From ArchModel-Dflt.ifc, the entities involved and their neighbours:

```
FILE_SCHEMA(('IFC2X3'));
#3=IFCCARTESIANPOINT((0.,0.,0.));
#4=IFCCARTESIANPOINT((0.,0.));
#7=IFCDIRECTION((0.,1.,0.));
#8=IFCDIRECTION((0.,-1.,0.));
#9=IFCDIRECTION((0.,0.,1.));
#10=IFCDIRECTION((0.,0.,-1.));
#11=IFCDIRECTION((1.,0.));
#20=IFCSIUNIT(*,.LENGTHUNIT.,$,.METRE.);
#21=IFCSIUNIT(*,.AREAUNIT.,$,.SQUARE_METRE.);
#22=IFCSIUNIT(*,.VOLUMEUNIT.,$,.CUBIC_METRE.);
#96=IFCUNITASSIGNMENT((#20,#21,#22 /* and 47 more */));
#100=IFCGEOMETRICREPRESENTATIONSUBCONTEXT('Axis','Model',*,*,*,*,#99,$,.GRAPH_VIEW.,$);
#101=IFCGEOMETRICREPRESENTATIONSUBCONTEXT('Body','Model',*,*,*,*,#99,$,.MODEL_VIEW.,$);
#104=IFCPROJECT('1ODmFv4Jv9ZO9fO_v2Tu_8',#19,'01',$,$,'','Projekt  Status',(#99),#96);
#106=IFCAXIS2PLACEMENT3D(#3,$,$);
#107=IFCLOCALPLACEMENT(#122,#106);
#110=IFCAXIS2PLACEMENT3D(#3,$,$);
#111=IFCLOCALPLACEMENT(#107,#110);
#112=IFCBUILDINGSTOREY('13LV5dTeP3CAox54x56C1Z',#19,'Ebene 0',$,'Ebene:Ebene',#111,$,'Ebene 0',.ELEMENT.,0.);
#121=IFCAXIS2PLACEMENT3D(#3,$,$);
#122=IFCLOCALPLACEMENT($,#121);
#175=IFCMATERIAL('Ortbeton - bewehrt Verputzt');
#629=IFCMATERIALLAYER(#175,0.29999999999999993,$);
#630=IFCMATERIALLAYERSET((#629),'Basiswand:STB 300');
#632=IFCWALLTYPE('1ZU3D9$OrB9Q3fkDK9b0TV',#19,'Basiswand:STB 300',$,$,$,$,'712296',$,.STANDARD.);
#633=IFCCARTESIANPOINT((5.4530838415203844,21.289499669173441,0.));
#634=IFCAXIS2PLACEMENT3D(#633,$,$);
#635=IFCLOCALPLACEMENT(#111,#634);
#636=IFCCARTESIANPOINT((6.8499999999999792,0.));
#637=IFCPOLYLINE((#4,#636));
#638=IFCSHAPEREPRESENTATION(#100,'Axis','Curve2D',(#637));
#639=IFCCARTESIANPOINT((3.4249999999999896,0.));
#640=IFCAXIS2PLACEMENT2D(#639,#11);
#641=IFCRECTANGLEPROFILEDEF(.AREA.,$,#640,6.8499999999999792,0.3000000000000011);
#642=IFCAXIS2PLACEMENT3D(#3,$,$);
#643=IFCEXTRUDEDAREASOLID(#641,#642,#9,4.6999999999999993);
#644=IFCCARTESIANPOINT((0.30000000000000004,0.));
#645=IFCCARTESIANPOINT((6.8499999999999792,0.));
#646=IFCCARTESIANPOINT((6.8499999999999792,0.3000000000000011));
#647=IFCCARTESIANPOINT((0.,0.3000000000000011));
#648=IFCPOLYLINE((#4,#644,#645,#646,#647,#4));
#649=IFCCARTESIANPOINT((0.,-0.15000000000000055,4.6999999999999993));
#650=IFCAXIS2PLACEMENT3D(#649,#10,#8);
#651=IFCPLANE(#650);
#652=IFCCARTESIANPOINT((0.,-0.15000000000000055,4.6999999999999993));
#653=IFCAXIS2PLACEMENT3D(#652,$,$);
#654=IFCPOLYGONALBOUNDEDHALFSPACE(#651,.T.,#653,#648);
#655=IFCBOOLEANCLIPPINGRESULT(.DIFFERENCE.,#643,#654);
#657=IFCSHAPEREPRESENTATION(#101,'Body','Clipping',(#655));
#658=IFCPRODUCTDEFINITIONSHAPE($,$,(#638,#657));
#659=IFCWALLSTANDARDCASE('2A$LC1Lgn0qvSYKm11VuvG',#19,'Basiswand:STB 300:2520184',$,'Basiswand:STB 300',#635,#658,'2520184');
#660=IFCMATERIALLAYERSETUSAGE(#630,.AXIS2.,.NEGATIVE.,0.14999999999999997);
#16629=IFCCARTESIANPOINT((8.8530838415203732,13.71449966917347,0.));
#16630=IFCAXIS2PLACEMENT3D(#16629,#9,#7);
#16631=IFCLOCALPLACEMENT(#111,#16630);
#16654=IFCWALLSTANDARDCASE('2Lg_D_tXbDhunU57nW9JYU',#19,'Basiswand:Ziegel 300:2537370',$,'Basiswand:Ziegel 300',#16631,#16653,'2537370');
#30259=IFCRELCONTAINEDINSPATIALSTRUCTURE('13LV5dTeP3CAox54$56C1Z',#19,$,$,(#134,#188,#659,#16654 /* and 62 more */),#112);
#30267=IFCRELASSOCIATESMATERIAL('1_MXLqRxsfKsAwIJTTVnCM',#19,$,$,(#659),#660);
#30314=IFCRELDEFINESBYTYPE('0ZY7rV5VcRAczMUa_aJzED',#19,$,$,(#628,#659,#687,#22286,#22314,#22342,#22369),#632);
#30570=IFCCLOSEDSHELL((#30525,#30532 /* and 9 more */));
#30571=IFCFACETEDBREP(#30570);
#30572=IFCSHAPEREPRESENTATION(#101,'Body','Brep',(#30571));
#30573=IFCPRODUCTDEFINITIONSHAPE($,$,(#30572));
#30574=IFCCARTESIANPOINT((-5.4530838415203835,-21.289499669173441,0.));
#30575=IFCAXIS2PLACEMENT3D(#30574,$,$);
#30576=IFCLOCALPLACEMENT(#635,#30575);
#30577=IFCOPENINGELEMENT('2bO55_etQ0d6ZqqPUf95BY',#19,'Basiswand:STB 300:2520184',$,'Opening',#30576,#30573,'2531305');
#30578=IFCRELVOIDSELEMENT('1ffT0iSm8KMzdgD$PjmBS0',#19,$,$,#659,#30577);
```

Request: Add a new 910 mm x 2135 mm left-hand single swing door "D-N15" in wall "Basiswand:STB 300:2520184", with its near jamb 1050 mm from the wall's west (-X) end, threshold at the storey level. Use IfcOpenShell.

```python
import numpy as np
import ifcopenshell
import ifcopenshell.api.feature
import ifcopenshell.api.geometry
import ifcopenshell.api.root
import ifcopenshell.api.spatial
import ifcopenshell.api.type
import ifcopenshell.geom
import ifcopenshell.util.element
import ifcopenshell.util.placement
import ifcopenshell.util.representation
import ifcopenshell.util.shape
import ifcopenshell.util.unit

model = ifcopenshell.open("ArchModel-Dflt.ifc")
unit_scale = ifcopenshell.util.unit.calculate_unit_scale(model)
settings = ifcopenshell.geom.settings()


def volume(element):
    """Net volume in cubic metres, openings subtracted."""
    shape = ifcopenshell.geom.create_shape(settings, element)
    return ifcopenshell.util.shape.get_volume(shape.geometry)


wall = model.by_guid("2A$LC1Lgn0qvSYKm11VuvG")
storey = ifcopenshell.util.element.get_container(wall, ifc_class="IfcBuildingStorey")
context = ifcopenshell.util.representation.get_context(model, "Model", "Body", "MODEL_VIEW")
before = volume(wall)

width, height, from_end, sill = 0.91, 2.135, 1.05, 0.0  # metres

# The wall runs along its own X axis, and the end named is its -X end.
wall_shape = ifcopenshell.geom.create_shape(settings, wall)
x, y, z = ifcopenshell.util.shape.get_vertices(wall_shape.geometry).T
start = x.min() + from_end
face, thickness = float(y.min()), float(y.max() - y.min())
wall_matrix = ifcopenshell.util.placement.get_local_placement(wall.ObjectPlacement)
level = ifcopenshell.util.placement.get_local_placement(storey.ObjectPlacement)[2, 3]


def in_wall(x, y):
    """Placement at x, y metres in the wall's axes, at sill height."""
    matrix = wall_matrix.copy()
    matrix[:, 3] = wall_matrix @ np.array([x / unit_scale, y / unit_scale, 0.0, 1.0])
    matrix[2, 3] = level + sill / unit_scale
    return matrix


# Opening: a box that overshoots both wall faces by 50 mm.
opening = ifcopenshell.api.root.create_entity(model, ifc_class="IfcOpeningElement")
box = ifcopenshell.api.geometry.add_wall_representation(
    model, context=context, length=width, height=height, thickness=thickness + 0.1
)
ifcopenshell.api.geometry.assign_representation(model, product=opening, representation=box)
ifcopenshell.api.geometry.edit_object_placement(model, product=opening, matrix=in_wall(start, face - 0.05), is_si=False)
ifcopenshell.api.feature.add_feature(model, feature=opening, element=wall)

door = ifcopenshell.api.root.create_entity(model, ifc_class="IfcDoor", name="D-N15")
door.OverallWidth, door.OverallHeight = width / unit_scale, height / unit_scale
body = ifcopenshell.api.geometry.add_door_representation(
    model,
    context=context,
    overall_width=door.OverallWidth,
    overall_height=door.OverallHeight,
    operation_type="SINGLE_SWING_LEFT",
    lining_properties={"LiningDepth": thickness / unit_scale, "ThresholdDepth": thickness / unit_scale},
)
ifcopenshell.api.geometry.assign_representation(model, product=door, representation=body)
ifcopenshell.api.spatial.assign_container(model, products=[door], relating_structure=storey)
fills = ifcopenshell.api.feature.add_filling(model, opening=opening, element=door)
fills.OwnerHistory = door.OwnerHistory  # required in IFC2X3

# IFC2X3 keeps the operation on the door style.
style = ifcopenshell.api.root.create_entity(model, ifc_class="IfcDoorStyle", name="D-N15")
style.OperationType, style.ConstructionType = "SINGLE_SWING_LEFT", "NOTDEFINED"
style.ParameterTakesPrecedence = style.Sizeable = False
ifcopenshell.api.type.assign_type(model, related_objects=[door], relating_type=style)

# The lining spans the wall, so the door starts at the wall face.
ifcopenshell.api.geometry.edit_object_placement(model, product=door, matrix=in_wall(start, face), is_si=False)

after = volume(wall)

print(f"wall volume {before:.3f} -> {after:.3f} m3")

model.write("ArchModel-Dflt-out.ifc")
```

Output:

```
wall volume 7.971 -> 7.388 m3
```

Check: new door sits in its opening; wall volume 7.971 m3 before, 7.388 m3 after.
